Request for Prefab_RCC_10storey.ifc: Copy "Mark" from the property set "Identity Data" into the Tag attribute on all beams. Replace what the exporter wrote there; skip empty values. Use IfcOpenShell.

First a look at what the model holds.

```python
import ifcopenshell
import ifcopenshell.util.element

model = ifcopenshell.open("Prefab_RCC_10storey.ifc")
print(model.schema)
beams = model.by_type("IfcBeam")
print(len(beams), "beams")
for e in beams[:8]:
    source = ifcopenshell.util.element.get_pset(e, "Identity Data", "Mark")
    target = e.Tag
    print(e.id(), repr(source), repr(target), sep=" | ")
```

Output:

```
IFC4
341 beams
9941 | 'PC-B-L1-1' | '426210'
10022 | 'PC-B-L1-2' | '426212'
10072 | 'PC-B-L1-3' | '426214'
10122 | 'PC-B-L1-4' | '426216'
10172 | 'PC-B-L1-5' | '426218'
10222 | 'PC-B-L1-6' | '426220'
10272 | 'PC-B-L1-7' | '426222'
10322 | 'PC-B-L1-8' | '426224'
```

```python
import ifcopenshell
import ifcopenshell.util.element

model = ifcopenshell.open("Prefab_RCC_10storey.ifc")

count = 0
for e in model.by_type("IfcBeam"):
    value = ifcopenshell.util.element.get_pset(e, "Identity Data", "Mark")
    current = e.Tag
    if not value or not value.strip() or current == value:
        continue
    e.Tag = value
    count += 1

print(count, "beams updated")

model.write("Prefab_RCC_10storey_updated.ifc")
```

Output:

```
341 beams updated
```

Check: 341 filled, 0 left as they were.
